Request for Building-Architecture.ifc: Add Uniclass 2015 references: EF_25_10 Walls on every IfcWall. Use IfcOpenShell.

First a look at what the model holds.

```python
import ifcopenshell

model = ifcopenshell.open("Building-Architecture.ifc")
print(model.schema)
print("classifications:", [c.Name for c in model.by_type("IfcClassification")])
for ifc_class in ("IfcDoor", "IfcRoof", "IfcStair", "IfcWall", "IfcWindow"):
    print(ifc_class, len(model.by_type(ifc_class)))
```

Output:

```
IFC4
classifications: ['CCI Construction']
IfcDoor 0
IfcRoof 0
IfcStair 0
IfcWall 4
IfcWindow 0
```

```python
import ifcopenshell
import ifcopenshell.api.classification

model = ifcopenshell.open("Building-Architecture.ifc")

system = ifcopenshell.api.classification.add_classification(model, classification="Uniclass 2015")

codes = {
    "IfcWall": ("EF_25_10", "Walls"),
}
for ifc_class, (code, name) in codes.items():
    products = model.by_type(ifc_class)
    ifcopenshell.api.classification.add_reference(
        model, products=products, classification=system, identification=code, name=name
    )
    print(code, len(products))

model.write("Building-Architecture_edited.ifc")
```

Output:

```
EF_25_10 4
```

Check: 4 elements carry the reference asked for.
